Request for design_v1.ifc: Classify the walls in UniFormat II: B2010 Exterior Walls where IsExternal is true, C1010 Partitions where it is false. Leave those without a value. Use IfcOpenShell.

First a look at what the model holds.

```python
import ifcopenshell
import ifcopenshell.util.element

model = ifcopenshell.open("design_v1.ifc")
print(model.schema)
print("classifications:", [c.Name for c in model.by_type("IfcClassification")])
values = [ifcopenshell.util.element.get_pset(e, "Pset_WallCommon", "IsExternal") for e in model.by_type("IfcWall")]
for value in (True, False, None):
    print("IsExternal", value, values.count(value))
```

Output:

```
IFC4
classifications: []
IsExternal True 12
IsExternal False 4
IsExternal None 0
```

```python
import ifcopenshell
import ifcopenshell.api.classification
import ifcopenshell.util.element

model = ifcopenshell.open("design_v1.ifc")

system = ifcopenshell.api.classification.add_classification(model, classification="UniFormat II")

walls = model.by_type("IfcWall")
external = {e: ifcopenshell.util.element.get_pset(e, "Pset_WallCommon", "IsExternal") for e in walls}
for flag, code, name in ((True, "B2010", "Exterior Walls"), (False, "C1010", "Partitions")):
    products = [e for e in walls if external[e] is flag]
    ifcopenshell.api.classification.add_reference(
        model, products=products, classification=system, identification=code, name=name
    )
    print(code, len(products))

model.write("design_v1-out.ifc")
```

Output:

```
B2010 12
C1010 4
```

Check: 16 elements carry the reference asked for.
